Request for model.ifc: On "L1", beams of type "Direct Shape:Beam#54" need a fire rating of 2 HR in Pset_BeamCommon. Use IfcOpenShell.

First a look at what the model holds.

```python
import ifcopenshell
import ifcopenshell.util.element

model = ifcopenshell.open("model.ifc")
print(model.schema)
storey = next(s for s in model.by_type("IfcBuildingStorey") if s.Name == "L1")
beams = [e for e in ifcopenshell.util.element.get_decomposition(storey) if e.is_a("IfcBeam")]
seen = {}
for e in beams:
    element_type = ifcopenshell.util.element.get_type(e)
    key = (element_type.Name if element_type != e and element_type else None, ifcopenshell.util.element.get_pset(e, "Pset_BeamCommon", "FireRating"))
    seen[key] = seen.get(key, 0) + 1
for (name, value), count in sorted(seen.items(), key=str):
    print(count, "x", name, "|", value)
```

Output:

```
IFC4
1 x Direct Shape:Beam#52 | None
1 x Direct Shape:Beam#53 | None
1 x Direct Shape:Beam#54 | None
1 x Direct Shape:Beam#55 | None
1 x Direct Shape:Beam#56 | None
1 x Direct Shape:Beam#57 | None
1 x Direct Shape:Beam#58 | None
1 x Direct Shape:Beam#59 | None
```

```python
import ifcopenshell
import ifcopenshell.api.pset
import ifcopenshell.util.element

model = ifcopenshell.open("model.ifc")

storey = next(s for s in model.by_type("IfcBuildingStorey") if s.Name == "L1")
beams = [e for e in ifcopenshell.util.element.get_decomposition(storey) if e.is_a("IfcBeam")]

count = 0
for e in beams:
    element_type = ifcopenshell.util.element.get_type(e)
    if element_type in (None, e) or element_type.Name != "Direct Shape:Beam#54":
        continue
    # add_pset returns the element's existing set when there is one.
    pset = ifcopenshell.api.pset.add_pset(model, product=e, name="Pset_BeamCommon")
    ifcopenshell.api.pset.edit_pset(model, pset=pset, properties={"FireRating": "2 HR"})
    count += 1

print(count, "beams updated")

model.write("model_v2.ifc")
```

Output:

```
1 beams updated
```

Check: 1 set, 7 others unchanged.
